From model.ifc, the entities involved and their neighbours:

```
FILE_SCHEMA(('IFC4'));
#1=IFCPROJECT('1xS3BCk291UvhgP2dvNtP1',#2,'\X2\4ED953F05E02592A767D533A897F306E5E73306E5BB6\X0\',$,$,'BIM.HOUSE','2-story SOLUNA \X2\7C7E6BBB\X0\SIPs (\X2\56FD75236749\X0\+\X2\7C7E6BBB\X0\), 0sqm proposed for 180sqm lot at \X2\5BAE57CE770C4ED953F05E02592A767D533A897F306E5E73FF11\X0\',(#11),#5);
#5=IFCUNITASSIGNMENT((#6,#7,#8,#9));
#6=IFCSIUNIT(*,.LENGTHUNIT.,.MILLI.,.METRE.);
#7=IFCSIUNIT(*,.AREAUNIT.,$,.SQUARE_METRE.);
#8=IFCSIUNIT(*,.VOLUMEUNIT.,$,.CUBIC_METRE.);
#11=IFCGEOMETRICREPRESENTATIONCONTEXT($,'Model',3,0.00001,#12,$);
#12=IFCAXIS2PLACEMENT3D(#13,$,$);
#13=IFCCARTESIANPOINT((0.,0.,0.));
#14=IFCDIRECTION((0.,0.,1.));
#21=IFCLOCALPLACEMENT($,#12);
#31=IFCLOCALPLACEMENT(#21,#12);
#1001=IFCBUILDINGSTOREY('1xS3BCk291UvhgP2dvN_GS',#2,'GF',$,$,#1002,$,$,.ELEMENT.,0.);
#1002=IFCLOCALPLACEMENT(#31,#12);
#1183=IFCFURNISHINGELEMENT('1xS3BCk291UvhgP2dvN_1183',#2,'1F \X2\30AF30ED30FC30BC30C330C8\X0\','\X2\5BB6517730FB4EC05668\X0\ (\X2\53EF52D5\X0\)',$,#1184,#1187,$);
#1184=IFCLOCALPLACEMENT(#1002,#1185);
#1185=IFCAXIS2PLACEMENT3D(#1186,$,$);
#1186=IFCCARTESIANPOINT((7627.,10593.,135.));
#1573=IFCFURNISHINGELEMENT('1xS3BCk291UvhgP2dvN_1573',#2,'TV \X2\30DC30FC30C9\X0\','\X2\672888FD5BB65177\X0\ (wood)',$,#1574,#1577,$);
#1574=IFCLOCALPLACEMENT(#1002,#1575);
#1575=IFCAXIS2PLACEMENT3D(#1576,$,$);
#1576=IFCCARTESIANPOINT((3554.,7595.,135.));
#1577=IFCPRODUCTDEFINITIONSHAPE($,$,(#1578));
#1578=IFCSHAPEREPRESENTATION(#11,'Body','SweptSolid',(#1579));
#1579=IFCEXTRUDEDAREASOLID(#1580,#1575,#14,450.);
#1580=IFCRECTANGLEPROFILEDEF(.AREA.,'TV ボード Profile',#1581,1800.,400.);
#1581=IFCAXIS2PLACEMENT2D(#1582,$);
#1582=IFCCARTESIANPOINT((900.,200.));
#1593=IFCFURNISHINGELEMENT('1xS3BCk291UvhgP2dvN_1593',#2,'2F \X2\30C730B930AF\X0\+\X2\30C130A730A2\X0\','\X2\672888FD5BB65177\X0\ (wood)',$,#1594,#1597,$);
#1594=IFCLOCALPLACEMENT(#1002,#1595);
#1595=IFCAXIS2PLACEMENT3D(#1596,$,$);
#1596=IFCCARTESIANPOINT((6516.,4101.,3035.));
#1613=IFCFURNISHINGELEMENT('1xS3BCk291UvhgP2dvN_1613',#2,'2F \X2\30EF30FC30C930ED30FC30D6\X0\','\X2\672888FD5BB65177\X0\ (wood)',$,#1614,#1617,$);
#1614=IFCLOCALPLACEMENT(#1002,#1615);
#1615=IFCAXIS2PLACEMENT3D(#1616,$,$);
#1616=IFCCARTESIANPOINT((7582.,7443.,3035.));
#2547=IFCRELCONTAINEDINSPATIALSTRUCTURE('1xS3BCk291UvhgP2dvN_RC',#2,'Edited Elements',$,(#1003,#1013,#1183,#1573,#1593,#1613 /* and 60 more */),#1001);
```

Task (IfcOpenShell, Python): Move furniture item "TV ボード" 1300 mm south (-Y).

```python
import ifcopenshell
import ifcopenshell.api.geometry
import ifcopenshell.util.placement
import ifcopenshell.util.unit

model = ifcopenshell.open("model.ifc")
unit_scale = ifcopenshell.util.unit.calculate_unit_scale(model)

item = model.by_guid("1xS3BCk291UvhgP2dvN_1573")
matrix = ifcopenshell.util.placement.get_local_placement(item.ObjectPlacement)
matrix[1, 3] -= 1.3 / unit_scale
ifcopenshell.api.geometry.edit_object_placement(model, product=item, matrix=matrix, is_si=False)

print(ifcopenshell.util.placement.get_local_placement(item.ObjectPlacement).round(3) + 0.0)

model.write("model_updated.ifc")
```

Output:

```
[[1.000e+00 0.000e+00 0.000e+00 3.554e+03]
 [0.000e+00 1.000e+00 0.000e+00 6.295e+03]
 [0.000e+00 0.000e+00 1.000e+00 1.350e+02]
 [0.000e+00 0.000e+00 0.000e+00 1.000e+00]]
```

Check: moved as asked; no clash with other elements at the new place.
